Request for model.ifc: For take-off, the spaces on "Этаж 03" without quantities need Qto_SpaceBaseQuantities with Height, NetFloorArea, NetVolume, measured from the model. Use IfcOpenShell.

First a look at what the model holds.

```python
import ifcopenshell
import ifcopenshell.util.element
import ifcopenshell.util.unit

model = ifcopenshell.open("model.ifc")
print(model.schema)
for unit_type in ("LENGTHUNIT", "AREAUNIT", "VOLUMEUNIT"):
    print(unit_type, ifcopenshell.util.unit.calculate_unit_scale(model, unit_type))
storey = next(s for s in model.by_type("IfcBuildingStorey") if s.Name == "Этаж 03")
spaces = [e for e in ifcopenshell.util.element.get_decomposition(storey) if e.is_a("IfcSpace")]
for e in sorted(spaces, key=lambda e: e.id()):
    print(e.id(), e.is_a(), e.Name, list(ifcopenshell.util.element.get_psets(e, qtos_only=True)), sep=" | ")
```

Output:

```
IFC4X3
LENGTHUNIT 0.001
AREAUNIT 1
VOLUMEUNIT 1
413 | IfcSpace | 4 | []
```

```python
import ifcopenshell
import ifcopenshell.api.pset
import ifcopenshell.geom
import ifcopenshell.util.element
import ifcopenshell.util.shape
import ifcopenshell.util.unit

model = ifcopenshell.open("model.ifc")
unit_scale = ifcopenshell.util.unit.calculate_unit_scale(model)
area_scale = ifcopenshell.util.unit.calculate_unit_scale(model, "AREAUNIT")
volume_scale = ifcopenshell.util.unit.calculate_unit_scale(model, "VOLUMEUNIT")
settings = ifcopenshell.geom.settings()

storey = next(s for s in model.by_type("IfcBuildingStorey") if s.Name == "Этаж 03")
spaces = [e for e in ifcopenshell.util.element.get_decomposition(storey) if e.is_a("IfcSpace")]

for e in sorted(spaces, key=lambda e: e.id()):
    if ifcopenshell.util.element.get_psets(e, qtos_only=True, should_inherit=False):
        continue
    # Geometry comes back in metres, in the element's own axes.
    shape = ifcopenshell.geom.create_shape(settings, e)
    values = {
        "Height": ifcopenshell.util.shape.get_z(shape.geometry) / unit_scale,
        "NetFloorArea": ifcopenshell.util.shape.get_footprint_area(shape.geometry) / area_scale,
        "NetVolume": ifcopenshell.util.shape.get_volume(shape.geometry) / volume_scale,
    }
    qto = ifcopenshell.api.pset.add_qto(model, product=e, name="Qto_SpaceBaseQuantities")
    ifcopenshell.api.pset.edit_qto(model, qto=qto, properties=values)
    print(e.id(), {k: round(v, 3) for k, v in values.items()})

model.write("model_updated.ifc")
```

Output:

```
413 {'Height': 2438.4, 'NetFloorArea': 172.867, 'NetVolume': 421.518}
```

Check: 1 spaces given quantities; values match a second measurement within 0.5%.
